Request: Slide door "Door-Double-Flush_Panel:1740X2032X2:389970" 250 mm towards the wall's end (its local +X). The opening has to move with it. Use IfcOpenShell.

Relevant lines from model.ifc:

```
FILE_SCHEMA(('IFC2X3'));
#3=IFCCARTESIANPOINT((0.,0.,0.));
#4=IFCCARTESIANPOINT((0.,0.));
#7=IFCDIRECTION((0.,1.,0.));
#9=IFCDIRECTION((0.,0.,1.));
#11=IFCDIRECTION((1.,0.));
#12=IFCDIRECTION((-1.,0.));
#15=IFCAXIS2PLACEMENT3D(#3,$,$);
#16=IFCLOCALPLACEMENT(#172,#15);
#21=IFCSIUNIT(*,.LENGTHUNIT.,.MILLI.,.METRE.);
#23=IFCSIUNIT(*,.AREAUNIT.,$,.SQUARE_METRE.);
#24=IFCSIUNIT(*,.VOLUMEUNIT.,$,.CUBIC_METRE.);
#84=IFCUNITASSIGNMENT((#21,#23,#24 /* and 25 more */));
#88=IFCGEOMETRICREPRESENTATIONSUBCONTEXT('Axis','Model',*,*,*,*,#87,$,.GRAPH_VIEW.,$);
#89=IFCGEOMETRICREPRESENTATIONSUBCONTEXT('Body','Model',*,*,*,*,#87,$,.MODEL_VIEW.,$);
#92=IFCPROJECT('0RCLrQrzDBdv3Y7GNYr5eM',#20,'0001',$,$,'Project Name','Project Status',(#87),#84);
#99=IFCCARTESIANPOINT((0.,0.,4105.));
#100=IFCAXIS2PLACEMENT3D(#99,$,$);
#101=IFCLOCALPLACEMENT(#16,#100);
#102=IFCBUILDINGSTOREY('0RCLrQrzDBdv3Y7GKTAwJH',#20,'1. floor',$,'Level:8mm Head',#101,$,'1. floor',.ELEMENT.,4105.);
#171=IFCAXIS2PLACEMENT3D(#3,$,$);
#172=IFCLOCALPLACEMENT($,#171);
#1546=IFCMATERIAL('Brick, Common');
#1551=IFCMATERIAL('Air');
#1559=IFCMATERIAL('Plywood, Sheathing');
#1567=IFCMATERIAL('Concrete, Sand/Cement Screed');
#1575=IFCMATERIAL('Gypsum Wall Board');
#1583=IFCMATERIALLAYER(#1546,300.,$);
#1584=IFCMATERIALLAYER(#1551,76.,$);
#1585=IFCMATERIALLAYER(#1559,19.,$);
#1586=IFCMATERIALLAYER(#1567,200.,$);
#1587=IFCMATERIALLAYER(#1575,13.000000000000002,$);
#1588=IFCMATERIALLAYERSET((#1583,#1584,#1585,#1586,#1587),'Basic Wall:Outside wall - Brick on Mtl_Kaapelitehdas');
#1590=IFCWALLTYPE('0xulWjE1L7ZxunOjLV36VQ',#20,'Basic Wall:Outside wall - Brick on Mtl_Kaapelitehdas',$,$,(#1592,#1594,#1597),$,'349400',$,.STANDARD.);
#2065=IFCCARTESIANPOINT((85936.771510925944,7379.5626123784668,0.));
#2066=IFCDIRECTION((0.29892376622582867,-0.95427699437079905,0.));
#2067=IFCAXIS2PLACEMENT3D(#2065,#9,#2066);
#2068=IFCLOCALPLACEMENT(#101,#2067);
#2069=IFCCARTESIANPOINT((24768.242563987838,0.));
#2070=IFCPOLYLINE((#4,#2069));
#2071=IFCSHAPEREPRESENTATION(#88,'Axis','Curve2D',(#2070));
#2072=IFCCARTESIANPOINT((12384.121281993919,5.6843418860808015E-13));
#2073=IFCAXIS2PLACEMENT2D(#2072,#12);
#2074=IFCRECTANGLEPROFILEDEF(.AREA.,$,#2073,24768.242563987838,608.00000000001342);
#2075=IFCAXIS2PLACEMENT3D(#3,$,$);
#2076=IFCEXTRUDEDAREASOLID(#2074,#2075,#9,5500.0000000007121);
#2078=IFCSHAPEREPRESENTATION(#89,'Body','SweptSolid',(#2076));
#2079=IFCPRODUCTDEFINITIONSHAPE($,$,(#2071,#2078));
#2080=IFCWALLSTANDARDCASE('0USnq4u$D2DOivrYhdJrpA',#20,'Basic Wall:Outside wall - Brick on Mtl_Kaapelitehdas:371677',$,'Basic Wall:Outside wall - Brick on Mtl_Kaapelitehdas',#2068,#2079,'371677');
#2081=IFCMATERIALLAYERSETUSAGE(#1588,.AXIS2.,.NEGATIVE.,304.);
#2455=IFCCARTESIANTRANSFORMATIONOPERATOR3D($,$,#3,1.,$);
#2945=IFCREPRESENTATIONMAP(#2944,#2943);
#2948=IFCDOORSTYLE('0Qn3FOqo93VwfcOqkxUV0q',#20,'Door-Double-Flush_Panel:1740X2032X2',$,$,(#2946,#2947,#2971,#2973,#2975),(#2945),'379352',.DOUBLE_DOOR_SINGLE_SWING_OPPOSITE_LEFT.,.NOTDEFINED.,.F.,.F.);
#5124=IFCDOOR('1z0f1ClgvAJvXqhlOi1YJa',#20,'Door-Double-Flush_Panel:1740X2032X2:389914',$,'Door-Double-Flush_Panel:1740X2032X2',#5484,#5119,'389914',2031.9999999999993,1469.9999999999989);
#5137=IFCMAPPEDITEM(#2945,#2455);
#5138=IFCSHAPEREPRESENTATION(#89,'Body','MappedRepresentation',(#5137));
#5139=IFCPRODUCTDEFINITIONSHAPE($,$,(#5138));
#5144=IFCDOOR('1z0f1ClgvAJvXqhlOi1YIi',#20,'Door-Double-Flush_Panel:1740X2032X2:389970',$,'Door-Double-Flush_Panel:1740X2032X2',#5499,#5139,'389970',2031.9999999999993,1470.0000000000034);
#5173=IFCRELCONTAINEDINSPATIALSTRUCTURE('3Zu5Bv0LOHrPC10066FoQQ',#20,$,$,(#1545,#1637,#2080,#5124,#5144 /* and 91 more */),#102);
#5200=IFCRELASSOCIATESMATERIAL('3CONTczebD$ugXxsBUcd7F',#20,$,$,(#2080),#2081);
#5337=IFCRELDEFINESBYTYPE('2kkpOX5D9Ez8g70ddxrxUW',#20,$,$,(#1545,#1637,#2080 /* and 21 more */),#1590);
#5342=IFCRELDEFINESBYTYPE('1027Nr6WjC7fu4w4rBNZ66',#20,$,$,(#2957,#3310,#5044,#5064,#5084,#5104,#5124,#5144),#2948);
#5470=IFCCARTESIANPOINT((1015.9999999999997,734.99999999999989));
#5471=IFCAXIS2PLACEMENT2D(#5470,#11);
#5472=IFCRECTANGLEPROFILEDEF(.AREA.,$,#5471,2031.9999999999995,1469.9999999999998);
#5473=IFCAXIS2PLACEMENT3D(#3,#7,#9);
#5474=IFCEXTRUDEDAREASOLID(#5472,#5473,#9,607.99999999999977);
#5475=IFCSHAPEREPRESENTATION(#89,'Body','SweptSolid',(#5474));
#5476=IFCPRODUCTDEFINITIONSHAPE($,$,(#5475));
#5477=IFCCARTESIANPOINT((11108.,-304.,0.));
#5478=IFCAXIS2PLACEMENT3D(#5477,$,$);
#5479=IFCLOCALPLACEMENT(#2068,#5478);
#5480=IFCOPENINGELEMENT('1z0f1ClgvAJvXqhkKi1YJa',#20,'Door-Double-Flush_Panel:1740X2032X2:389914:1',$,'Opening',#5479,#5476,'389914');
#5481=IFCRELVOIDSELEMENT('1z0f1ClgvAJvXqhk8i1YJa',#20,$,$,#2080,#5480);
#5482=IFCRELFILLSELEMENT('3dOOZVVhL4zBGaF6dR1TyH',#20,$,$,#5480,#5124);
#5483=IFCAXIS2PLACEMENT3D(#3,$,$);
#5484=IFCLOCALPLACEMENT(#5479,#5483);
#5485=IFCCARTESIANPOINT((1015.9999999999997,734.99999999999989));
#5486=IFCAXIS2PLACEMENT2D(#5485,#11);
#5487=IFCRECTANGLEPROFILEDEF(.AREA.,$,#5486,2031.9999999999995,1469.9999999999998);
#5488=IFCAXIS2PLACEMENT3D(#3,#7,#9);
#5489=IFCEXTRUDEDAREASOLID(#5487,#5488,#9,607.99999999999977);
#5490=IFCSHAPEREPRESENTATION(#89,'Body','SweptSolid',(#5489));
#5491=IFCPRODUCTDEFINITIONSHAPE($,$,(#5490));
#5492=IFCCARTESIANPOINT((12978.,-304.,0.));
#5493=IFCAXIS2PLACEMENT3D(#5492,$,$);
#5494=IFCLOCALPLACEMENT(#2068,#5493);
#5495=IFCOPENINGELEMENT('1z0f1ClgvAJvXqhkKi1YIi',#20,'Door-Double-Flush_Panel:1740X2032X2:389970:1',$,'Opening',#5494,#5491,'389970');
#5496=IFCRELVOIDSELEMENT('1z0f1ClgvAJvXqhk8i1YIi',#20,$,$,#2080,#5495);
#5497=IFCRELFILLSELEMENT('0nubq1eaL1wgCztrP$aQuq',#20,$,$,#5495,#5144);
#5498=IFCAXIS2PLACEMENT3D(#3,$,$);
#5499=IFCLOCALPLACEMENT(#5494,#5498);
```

```python
import ifcopenshell
import ifcopenshell.api.geometry
import ifcopenshell.util.placement

model = ifcopenshell.open("model.ifc")

door = model.by_guid("1z0f1ClgvAJvXqhlOi1YIi")
opening = door.FillsVoids[0].RelatingOpeningElement
wall = opening.VoidsElements[0].RelatingBuildingElement

wall_matrix = ifcopenshell.util.placement.get_local_placement(wall.ObjectPlacement)
shift = wall_matrix[:3, 0] * 250.0
before = ifcopenshell.util.placement.get_local_placement(door.ObjectPlacement)[:3, 3].copy()

# The door is placed relative to its opening, so it follows when the opening moves.
matrix = ifcopenshell.util.placement.get_local_placement(opening.ObjectPlacement)
matrix[:3, 3] += shift
ifcopenshell.api.geometry.edit_object_placement(
    model, product=opening, matrix=matrix, is_si=False, should_transform_children=True
)

after = ifcopenshell.util.placement.get_local_placement(door.ObjectPlacement)[:3, 3]
print("door moved by", (after - before).round(3) + 0.0)

model.write("model_edited.ifc")
```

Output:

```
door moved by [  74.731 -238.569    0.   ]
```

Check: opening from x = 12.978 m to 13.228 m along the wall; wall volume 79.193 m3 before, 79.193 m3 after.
